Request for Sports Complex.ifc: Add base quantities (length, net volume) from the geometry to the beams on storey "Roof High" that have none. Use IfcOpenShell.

First a look at what the model holds.

```python
import ifcopenshell
import ifcopenshell.util.element
import ifcopenshell.util.unit

model = ifcopenshell.open("Sports Complex.ifc")
print(model.schema)
for unit_type in ("LENGTHUNIT", "AREAUNIT", "VOLUMEUNIT"):
    print(unit_type, ifcopenshell.util.unit.calculate_unit_scale(model, unit_type))
storey = next(s for s in model.by_type("IfcBuildingStorey") if s.Name == "Roof High")
beams = [e for e in ifcopenshell.util.element.get_decomposition(storey) if e.is_a("IfcBeam")]
for e in sorted(beams, key=lambda e: e.id()):
    print(e.id(), e.is_a(), e.Name, list(ifcopenshell.util.element.get_psets(e, qtos_only=True)), sep=" | ")
```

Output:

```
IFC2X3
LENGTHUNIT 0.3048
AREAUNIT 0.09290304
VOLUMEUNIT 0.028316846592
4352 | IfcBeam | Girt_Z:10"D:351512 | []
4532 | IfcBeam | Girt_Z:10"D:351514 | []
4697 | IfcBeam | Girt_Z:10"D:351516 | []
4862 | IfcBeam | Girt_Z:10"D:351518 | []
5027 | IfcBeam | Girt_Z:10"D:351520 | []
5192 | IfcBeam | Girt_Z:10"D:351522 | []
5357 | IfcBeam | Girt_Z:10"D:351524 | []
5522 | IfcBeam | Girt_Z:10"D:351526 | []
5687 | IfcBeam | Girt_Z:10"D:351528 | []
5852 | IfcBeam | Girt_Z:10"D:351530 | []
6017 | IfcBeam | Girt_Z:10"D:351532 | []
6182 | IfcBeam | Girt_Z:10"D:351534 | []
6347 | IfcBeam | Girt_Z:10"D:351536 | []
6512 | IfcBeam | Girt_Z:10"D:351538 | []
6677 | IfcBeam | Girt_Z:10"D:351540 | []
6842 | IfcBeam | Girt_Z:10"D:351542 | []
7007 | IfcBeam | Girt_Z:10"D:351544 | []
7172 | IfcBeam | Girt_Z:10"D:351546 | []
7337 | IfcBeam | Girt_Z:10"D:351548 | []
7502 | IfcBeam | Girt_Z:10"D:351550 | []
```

```python
import ifcopenshell
import ifcopenshell.api.pset
import ifcopenshell.geom
import ifcopenshell.util.element
import ifcopenshell.util.shape
import ifcopenshell.util.unit

model = ifcopenshell.open("Sports Complex.ifc")
unit_scale = ifcopenshell.util.unit.calculate_unit_scale(model)
volume_scale = ifcopenshell.util.unit.calculate_unit_scale(model, "VOLUMEUNIT")
settings = ifcopenshell.geom.settings()

storey = next(s for s in model.by_type("IfcBuildingStorey") if s.Name == "Roof High")
beams = [e for e in ifcopenshell.util.element.get_decomposition(storey) if e.is_a("IfcBeam")]

for e in sorted(beams, key=lambda e: e.id()):
    if ifcopenshell.util.element.get_psets(e, qtos_only=True, should_inherit=False):
        continue
    # Geometry comes back in metres, in the element's own axes.
    shape = ifcopenshell.geom.create_shape(settings, e)
    values = {
        "Length": ifcopenshell.util.shape.get_max_xyz(shape.geometry) / unit_scale,
        "NetVolume": ifcopenshell.util.shape.get_volume(shape.geometry) / volume_scale,
    }
    qto = ifcopenshell.api.pset.add_qto(model, product=e, name="BaseQuantities")
    ifcopenshell.api.pset.edit_qto(model, qto=qto, properties=values)
    print(e.id(), {k: round(v, 3) for k, v in values.items()})

model.write("Sports Complex_rev.ifc")
```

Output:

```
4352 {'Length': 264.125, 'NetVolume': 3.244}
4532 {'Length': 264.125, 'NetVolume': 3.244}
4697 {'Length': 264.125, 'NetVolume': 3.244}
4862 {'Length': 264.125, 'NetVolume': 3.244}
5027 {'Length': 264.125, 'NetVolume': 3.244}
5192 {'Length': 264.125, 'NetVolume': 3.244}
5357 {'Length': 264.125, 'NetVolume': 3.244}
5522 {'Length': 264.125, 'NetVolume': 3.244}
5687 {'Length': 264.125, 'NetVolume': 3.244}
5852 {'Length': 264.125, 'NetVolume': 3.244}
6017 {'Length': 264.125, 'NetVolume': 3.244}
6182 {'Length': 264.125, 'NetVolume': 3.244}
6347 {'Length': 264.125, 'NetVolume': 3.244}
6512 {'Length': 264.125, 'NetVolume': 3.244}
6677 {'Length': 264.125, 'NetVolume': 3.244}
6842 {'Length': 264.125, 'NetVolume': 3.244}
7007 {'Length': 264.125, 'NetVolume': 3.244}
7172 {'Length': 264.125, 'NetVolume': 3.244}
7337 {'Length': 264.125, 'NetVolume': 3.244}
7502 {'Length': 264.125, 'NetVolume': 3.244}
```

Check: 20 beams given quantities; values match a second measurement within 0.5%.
